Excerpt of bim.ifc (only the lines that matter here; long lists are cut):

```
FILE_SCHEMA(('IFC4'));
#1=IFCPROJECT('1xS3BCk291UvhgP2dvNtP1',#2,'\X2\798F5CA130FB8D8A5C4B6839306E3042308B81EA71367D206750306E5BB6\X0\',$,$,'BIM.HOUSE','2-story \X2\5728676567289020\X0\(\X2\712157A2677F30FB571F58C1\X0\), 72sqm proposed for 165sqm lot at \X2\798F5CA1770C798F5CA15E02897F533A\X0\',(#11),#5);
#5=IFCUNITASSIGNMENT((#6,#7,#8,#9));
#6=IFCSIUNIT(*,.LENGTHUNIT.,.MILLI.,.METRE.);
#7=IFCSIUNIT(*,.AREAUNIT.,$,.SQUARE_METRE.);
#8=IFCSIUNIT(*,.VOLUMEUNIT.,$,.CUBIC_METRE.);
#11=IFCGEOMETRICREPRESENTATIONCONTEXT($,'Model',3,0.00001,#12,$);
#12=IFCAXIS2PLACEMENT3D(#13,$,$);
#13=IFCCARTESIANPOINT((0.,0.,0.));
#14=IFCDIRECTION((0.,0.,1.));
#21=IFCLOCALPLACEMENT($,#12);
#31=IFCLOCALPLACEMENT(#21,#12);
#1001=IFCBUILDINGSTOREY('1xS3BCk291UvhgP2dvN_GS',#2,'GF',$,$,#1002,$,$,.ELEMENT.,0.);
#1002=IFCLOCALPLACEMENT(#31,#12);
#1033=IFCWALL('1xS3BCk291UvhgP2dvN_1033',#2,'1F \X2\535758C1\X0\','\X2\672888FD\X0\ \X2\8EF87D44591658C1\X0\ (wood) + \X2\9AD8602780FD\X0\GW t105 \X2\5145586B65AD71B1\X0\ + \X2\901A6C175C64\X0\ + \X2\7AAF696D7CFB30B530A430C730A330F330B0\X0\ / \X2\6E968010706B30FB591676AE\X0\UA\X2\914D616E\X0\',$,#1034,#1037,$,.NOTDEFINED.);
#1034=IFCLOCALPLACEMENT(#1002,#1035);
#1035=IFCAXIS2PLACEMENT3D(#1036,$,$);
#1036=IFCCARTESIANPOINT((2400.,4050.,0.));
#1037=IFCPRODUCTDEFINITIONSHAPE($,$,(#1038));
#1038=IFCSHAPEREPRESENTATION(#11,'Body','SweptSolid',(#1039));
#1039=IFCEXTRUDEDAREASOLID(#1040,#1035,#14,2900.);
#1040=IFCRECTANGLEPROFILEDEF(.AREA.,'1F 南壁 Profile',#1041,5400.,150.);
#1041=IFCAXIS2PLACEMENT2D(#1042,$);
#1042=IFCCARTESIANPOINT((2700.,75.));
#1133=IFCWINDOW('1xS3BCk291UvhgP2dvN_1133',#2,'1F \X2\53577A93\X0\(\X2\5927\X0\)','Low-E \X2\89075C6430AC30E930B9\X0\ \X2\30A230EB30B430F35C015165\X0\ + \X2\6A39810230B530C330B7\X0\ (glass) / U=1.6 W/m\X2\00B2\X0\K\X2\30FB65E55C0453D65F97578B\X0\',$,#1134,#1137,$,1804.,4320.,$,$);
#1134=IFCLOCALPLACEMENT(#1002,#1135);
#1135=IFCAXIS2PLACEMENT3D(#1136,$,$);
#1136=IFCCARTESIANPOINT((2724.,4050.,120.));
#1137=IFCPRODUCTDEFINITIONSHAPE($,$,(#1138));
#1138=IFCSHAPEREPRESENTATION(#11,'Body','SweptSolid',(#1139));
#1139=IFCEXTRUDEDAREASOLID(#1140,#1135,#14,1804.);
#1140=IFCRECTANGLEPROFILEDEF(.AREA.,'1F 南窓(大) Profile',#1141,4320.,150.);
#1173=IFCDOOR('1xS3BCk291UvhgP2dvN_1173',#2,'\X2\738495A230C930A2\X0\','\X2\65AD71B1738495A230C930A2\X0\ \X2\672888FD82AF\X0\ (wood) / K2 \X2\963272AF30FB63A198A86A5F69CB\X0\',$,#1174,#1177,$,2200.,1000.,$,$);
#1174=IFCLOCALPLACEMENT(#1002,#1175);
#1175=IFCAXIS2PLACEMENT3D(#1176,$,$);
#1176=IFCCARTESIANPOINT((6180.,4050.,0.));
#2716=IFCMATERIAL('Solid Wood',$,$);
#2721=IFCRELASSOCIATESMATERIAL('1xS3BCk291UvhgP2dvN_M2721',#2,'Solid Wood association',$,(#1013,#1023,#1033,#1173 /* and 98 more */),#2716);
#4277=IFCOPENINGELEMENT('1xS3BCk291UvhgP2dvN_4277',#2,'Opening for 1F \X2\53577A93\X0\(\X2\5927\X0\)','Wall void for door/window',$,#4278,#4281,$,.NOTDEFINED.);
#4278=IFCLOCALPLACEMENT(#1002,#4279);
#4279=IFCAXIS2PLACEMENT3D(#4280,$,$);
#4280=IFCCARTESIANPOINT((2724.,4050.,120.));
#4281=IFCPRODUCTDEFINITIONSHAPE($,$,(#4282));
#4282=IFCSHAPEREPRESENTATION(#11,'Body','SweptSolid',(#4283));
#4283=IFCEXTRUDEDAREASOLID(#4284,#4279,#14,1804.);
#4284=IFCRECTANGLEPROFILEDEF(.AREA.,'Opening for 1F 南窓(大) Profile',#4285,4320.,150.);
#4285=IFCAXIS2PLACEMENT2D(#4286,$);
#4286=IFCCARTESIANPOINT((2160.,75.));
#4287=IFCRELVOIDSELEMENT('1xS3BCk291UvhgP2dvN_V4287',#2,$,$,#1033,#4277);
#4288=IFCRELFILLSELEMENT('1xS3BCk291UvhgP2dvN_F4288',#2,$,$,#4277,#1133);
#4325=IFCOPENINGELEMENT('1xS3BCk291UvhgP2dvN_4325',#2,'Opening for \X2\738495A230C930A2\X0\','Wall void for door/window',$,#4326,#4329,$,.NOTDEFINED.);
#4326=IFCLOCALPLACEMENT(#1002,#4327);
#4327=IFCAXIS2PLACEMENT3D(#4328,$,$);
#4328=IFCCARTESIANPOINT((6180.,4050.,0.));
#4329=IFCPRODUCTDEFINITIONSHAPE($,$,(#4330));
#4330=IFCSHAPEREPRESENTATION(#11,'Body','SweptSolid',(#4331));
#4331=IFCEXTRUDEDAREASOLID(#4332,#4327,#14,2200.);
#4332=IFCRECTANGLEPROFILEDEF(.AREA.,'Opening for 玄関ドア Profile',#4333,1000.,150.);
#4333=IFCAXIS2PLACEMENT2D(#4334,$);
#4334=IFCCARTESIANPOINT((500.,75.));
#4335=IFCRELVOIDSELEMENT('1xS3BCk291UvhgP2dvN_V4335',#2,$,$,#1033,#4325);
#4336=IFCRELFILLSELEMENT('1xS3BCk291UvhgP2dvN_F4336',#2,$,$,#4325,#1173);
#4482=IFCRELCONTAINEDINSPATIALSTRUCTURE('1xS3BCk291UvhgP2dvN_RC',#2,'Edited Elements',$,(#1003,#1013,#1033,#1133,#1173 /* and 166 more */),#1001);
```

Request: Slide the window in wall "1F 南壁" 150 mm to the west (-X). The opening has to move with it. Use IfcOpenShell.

```python
import ifcopenshell
import ifcopenshell.api.geometry
import ifcopenshell.util.placement
import ifcopenshell.util.unit

model = ifcopenshell.open("bim.ifc")
unit_scale = ifcopenshell.util.unit.calculate_unit_scale(model)

window = model.by_id(1133)
opening = window.FillsVoids[0].RelatingOpeningElement
wall = opening.VoidsElements[0].RelatingBuildingElement

wall_matrix = ifcopenshell.util.placement.get_local_placement(wall.ObjectPlacement)
shift = wall_matrix[:3, 0] * -0.15 / unit_scale
before = ifcopenshell.util.placement.get_local_placement(window.ObjectPlacement)[:3, 3].copy()

# The window is not placed relative to its opening, so move both.
for product in (opening, window):
    matrix = ifcopenshell.util.placement.get_local_placement(product.ObjectPlacement)
    matrix[:3, 3] += shift
    ifcopenshell.api.geometry.edit_object_placement(model, product=product, matrix=matrix, is_si=False)

after = ifcopenshell.util.placement.get_local_placement(window.ObjectPlacement)[:3, 3]
print("window moved by", (after - before).round(3) + 0.0)

model.write("bim_edited.ifc")
```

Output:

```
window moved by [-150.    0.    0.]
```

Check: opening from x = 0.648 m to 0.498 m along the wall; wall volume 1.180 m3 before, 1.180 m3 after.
